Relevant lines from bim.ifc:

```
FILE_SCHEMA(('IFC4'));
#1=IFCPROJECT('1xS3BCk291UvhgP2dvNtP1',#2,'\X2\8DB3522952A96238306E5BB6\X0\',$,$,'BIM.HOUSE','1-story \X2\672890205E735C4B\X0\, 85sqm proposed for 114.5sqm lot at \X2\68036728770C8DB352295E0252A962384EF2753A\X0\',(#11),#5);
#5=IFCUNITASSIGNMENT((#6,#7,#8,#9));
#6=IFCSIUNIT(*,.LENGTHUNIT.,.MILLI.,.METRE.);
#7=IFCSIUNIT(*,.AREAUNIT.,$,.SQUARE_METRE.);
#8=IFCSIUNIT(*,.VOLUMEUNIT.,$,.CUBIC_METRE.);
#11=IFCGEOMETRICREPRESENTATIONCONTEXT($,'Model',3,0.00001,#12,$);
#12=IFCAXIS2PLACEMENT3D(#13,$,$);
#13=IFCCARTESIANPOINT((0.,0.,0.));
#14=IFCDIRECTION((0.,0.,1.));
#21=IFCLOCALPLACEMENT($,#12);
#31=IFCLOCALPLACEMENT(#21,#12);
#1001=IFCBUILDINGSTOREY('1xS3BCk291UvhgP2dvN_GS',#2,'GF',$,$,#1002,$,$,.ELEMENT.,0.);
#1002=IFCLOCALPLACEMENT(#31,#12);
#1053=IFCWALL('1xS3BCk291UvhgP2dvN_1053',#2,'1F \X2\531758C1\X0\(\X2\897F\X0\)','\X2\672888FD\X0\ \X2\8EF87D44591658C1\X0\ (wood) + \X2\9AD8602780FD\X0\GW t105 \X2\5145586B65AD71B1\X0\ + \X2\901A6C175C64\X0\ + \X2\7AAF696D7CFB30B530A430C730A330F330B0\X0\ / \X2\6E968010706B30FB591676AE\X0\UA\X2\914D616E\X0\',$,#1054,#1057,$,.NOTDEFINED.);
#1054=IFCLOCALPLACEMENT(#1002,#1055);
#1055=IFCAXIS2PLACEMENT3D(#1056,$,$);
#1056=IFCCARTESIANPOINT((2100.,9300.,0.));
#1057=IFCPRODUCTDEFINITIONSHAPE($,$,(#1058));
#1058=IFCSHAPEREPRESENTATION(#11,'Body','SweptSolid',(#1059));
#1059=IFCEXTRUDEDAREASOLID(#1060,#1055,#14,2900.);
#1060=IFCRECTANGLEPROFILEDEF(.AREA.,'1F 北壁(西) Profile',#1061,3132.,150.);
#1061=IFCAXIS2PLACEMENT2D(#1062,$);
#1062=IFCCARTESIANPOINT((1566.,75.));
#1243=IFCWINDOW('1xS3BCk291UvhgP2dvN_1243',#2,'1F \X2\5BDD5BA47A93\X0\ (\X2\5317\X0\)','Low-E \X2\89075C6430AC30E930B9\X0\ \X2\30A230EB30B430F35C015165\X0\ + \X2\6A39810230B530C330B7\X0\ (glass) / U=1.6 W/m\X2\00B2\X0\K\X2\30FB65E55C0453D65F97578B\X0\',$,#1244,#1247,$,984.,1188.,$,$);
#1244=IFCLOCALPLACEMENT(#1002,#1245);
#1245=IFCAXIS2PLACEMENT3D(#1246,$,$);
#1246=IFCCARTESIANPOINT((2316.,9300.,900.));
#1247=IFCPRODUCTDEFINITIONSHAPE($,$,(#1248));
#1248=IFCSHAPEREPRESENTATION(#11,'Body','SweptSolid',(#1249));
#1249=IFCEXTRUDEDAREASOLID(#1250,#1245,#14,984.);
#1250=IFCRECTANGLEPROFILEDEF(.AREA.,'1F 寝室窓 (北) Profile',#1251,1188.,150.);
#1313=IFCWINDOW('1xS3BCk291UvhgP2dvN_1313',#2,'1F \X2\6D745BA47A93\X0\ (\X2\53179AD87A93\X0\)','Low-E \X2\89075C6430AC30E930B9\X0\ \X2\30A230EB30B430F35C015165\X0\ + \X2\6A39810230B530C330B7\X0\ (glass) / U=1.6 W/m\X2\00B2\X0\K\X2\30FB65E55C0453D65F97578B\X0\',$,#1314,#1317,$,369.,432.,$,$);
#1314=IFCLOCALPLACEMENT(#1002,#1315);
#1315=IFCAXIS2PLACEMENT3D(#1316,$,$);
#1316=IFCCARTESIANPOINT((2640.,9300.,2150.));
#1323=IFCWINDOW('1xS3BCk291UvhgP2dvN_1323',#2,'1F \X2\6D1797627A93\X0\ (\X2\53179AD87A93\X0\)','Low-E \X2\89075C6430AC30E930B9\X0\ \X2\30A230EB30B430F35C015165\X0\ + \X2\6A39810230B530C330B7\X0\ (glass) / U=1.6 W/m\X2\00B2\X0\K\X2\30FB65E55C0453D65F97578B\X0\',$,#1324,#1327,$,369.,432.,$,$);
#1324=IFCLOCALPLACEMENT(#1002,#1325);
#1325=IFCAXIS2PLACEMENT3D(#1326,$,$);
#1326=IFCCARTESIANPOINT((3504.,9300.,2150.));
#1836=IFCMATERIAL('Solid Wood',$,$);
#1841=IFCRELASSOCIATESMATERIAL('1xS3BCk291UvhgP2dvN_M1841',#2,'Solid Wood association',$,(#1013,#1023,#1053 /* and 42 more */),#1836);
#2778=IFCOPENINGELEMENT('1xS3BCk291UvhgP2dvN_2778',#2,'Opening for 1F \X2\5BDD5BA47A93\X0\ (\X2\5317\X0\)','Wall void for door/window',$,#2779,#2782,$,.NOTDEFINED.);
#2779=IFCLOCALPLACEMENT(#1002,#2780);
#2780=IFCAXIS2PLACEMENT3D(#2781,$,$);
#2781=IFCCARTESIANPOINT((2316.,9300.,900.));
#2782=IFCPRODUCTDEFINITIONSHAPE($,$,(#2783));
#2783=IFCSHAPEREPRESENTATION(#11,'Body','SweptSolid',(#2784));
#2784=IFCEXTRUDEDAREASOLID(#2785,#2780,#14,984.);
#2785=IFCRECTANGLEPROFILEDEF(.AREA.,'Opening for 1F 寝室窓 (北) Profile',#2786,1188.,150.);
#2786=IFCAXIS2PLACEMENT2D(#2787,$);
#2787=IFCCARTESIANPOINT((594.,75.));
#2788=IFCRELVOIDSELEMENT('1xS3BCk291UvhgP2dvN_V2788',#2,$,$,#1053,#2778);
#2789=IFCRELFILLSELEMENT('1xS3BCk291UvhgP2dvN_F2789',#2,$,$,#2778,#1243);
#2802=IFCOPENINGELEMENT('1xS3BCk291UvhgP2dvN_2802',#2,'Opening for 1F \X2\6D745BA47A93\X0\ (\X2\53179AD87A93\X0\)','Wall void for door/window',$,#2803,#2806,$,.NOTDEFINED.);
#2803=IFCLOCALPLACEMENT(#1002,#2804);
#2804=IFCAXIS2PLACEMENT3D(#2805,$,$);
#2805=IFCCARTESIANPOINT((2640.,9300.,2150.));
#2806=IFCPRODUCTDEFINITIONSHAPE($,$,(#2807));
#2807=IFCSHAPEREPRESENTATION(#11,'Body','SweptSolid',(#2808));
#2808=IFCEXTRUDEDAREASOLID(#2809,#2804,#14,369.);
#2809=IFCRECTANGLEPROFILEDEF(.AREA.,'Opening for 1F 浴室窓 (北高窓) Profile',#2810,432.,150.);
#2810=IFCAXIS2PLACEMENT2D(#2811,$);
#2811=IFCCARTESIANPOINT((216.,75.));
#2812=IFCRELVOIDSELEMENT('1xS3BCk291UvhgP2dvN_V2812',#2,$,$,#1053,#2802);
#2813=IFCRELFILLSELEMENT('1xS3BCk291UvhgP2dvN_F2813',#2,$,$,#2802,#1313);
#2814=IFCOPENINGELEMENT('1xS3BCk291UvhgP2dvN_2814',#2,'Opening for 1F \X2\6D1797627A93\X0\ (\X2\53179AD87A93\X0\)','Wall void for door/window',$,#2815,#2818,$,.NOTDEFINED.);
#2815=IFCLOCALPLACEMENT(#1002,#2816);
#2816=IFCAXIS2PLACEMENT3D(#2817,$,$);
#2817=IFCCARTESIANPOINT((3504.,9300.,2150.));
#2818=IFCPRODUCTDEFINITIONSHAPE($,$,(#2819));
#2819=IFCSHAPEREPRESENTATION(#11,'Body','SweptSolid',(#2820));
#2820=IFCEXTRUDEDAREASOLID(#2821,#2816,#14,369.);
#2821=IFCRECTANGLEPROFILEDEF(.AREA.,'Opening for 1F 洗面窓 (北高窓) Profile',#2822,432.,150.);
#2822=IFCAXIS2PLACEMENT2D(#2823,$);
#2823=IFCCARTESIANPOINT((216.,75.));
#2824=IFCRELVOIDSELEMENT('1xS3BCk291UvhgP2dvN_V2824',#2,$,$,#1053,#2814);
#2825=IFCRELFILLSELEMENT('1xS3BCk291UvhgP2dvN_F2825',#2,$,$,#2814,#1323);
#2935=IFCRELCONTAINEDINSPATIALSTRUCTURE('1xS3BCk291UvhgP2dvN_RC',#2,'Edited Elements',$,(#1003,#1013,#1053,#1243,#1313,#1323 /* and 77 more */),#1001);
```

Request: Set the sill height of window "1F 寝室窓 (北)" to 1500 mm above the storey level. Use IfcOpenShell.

```python
import numpy as np
import ifcopenshell
import ifcopenshell.api.geometry
import ifcopenshell.geom
import ifcopenshell.util.element
import ifcopenshell.util.placement
import ifcopenshell.util.shape
import ifcopenshell.util.unit

model = ifcopenshell.open("bim.ifc")
unit_scale = ifcopenshell.util.unit.calculate_unit_scale(model)

window = model.by_guid("1xS3BCk291UvhgP2dvN_1243")
opening = window.FillsVoids[0].RelatingOpeningElement
storey = ifcopenshell.util.element.get_container(window, ifc_class="IfcBuildingStorey")
level = ifcopenshell.util.placement.get_local_placement(storey.ObjectPlacement)[2, 3]

# The opening's origin need not be at the sill, so measure its lowest point.
shape = ifcopenshell.geom.create_shape(ifcopenshell.geom.settings(), opening)
bottom = ifcopenshell.util.shape.get_shape_bottom_elevation(shape, shape.geometry) / unit_scale
dz = level + 1.5 / unit_scale - bottom

shift = np.array([0.0, 0.0, dz])
# The window is not placed relative to its opening, so move both.
for product in (opening, window):
    matrix = ifcopenshell.util.placement.get_local_placement(product.ObjectPlacement)
    matrix[:3, 3] += shift
    ifcopenshell.api.geometry.edit_object_placement(model, product=product, matrix=matrix, is_si=False)

print(f"moved by {dz * unit_scale:+.3f} m")

model.write("bim_edited.ifc")
```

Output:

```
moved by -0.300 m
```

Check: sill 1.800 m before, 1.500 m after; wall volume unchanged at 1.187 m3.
